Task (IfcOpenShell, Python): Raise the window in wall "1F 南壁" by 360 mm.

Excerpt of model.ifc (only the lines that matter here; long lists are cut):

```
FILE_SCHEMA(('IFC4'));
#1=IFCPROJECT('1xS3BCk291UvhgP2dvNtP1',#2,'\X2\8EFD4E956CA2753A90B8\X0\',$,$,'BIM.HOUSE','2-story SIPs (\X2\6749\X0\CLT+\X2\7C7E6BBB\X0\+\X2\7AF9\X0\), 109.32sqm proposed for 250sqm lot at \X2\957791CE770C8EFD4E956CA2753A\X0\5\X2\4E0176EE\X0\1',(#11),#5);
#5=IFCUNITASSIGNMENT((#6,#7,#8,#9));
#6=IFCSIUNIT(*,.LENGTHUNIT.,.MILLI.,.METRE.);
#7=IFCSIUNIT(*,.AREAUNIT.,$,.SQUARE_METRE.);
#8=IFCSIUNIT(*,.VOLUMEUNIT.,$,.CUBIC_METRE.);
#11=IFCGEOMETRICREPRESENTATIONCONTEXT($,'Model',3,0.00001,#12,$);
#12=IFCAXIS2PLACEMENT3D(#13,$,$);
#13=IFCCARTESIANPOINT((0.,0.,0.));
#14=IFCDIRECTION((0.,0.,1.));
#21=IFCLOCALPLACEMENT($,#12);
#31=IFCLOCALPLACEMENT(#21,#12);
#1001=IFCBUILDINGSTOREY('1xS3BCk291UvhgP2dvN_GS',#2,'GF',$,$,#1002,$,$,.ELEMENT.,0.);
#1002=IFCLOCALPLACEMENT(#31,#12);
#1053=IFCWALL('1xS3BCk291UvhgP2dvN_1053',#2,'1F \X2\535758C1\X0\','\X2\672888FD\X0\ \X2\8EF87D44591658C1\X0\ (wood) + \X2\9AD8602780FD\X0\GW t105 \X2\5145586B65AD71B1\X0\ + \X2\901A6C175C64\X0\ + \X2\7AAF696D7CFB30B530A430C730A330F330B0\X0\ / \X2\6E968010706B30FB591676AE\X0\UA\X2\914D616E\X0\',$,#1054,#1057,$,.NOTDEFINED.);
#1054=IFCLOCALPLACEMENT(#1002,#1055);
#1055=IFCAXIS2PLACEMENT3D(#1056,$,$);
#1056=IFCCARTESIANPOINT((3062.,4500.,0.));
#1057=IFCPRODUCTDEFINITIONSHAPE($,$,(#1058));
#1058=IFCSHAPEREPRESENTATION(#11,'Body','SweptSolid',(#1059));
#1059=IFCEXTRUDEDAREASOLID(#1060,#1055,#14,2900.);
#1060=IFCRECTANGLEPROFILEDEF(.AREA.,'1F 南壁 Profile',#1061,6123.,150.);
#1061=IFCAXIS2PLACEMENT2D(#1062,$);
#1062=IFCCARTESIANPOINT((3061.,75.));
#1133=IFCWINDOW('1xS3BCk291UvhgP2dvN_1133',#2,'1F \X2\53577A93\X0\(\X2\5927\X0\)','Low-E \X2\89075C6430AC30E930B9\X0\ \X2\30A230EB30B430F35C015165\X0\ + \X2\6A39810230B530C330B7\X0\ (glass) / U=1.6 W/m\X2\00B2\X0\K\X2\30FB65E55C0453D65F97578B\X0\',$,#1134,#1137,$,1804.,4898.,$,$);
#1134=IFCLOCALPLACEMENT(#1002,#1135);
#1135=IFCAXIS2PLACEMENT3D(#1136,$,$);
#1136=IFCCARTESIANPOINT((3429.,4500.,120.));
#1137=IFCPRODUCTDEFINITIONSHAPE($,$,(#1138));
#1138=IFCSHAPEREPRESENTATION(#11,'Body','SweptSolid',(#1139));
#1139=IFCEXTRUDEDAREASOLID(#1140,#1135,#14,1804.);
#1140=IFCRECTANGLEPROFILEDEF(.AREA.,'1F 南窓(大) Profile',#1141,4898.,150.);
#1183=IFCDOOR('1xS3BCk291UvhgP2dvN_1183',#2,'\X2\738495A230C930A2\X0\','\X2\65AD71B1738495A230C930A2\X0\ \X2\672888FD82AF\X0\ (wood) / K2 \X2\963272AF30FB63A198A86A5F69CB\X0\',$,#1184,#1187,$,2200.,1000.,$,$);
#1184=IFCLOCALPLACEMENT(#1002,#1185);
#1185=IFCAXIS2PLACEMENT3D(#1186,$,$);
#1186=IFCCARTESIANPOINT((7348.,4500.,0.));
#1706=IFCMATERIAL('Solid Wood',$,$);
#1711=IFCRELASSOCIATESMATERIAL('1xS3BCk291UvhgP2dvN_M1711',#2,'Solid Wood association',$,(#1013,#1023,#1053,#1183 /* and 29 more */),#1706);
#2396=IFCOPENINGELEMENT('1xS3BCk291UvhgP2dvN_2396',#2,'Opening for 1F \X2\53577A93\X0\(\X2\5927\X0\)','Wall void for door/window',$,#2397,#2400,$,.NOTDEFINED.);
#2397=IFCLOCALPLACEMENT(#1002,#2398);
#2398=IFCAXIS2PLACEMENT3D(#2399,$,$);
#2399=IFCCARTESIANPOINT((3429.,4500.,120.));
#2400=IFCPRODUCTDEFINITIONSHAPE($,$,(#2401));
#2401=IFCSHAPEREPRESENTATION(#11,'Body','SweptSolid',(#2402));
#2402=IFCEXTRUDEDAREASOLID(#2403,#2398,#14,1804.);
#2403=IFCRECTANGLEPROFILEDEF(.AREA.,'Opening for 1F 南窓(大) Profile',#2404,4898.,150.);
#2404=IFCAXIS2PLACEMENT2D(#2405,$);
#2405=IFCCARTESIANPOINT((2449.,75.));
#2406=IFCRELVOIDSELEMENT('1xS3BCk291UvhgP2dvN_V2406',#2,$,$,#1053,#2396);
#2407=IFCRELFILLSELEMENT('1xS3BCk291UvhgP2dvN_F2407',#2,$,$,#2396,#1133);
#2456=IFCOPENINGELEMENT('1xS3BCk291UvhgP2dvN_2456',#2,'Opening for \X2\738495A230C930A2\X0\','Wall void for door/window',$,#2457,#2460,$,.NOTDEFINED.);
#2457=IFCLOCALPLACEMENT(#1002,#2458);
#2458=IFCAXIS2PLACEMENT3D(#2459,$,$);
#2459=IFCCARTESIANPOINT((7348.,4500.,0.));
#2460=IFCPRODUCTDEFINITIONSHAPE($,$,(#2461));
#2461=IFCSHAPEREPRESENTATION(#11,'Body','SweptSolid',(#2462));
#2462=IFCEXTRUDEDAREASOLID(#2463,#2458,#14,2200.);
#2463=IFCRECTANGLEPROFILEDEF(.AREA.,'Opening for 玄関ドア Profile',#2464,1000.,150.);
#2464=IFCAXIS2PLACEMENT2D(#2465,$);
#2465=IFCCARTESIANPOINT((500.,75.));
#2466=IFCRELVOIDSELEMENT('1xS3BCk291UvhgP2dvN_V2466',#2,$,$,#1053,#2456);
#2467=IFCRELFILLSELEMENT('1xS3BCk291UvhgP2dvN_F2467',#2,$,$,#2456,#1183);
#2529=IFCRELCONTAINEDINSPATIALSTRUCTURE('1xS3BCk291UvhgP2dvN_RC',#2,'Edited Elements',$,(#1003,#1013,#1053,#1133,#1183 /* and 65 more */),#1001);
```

```python
import numpy as np
import ifcopenshell
import ifcopenshell.api.geometry
import ifcopenshell.util.placement
import ifcopenshell.util.unit

model = ifcopenshell.open("model.ifc")
unit_scale = ifcopenshell.util.unit.calculate_unit_scale(model)

window = model.by_guid("1xS3BCk291UvhgP2dvN_1133")
opening = window.FillsVoids[0].RelatingOpeningElement
dz = 360.0

shift = np.array([0.0, 0.0, dz])
# The window is not placed relative to its opening, so move both.
for product in (opening, window):
    matrix = ifcopenshell.util.placement.get_local_placement(product.ObjectPlacement)
    matrix[:3, 3] += shift
    ifcopenshell.api.geometry.edit_object_placement(model, product=product, matrix=matrix, is_si=False)

print(f"moved by {dz * unit_scale:+.3f} m")

model.write("model_v2.ifc")
```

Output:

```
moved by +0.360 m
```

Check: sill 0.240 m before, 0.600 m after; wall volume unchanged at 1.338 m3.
